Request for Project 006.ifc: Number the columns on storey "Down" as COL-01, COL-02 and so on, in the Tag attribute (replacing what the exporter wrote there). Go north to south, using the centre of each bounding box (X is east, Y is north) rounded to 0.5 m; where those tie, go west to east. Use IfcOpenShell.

First a look at what the model holds.

```python
import ifcopenshell
import ifcopenshell.util.element
import ifcopenshell.util.placement

model = ifcopenshell.open("Project 006.ifc")
print(model.schema)
storey = next(s for s in model.by_type("IfcBuildingStorey") if s.Name == "Down")
columns = [e for e in ifcopenshell.util.element.get_decomposition(storey) if e.is_a("IfcColumn")]
for e in sorted(columns, key=lambda e: e.id()):
    origin = ifcopenshell.util.placement.get_local_placement(e.ObjectPlacement)[:3, 3]
    print(e.id(), e.Tag, e.Name, origin.round(2) + 0.0, sep=" | ")
```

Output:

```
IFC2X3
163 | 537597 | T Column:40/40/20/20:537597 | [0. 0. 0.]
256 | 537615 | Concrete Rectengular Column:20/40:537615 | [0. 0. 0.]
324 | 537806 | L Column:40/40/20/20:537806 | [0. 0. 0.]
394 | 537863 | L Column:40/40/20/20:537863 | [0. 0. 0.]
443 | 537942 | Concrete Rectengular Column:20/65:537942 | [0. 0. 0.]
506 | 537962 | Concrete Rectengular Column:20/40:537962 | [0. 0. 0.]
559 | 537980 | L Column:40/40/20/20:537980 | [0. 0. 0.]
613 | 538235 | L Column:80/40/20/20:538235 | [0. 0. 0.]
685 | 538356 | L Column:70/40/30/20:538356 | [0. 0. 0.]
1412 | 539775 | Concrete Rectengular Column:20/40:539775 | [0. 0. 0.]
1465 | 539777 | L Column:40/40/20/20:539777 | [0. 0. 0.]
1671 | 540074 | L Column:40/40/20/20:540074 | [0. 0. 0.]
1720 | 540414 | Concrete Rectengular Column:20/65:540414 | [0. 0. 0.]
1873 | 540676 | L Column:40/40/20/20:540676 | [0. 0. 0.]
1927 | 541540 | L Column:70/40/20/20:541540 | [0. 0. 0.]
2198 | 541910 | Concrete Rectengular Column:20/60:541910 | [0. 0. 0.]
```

```python
import ifcopenshell
import ifcopenshell.geom
import ifcopenshell.util.element
import ifcopenshell.util.shape

model = ifcopenshell.open("Project 006.ifc")
settings = ifcopenshell.geom.settings()
settings.set("use-world-coords", True)


def centre(element):
    shape = ifcopenshell.geom.create_shape(settings, element)
    return ifcopenshell.util.shape.get_bbox_centroid(shape.geometry)


storey = next(s for s in model.by_type("IfcBuildingStorey") if s.Name == "Down")
columns = [e for e in ifcopenshell.util.element.get_decomposition(storey) if e.is_a("IfcColumn")]

# Insertion points can sit at a corner or the storey origin, so sort by the geometry (in metres).
centres = {e: centre(e) for e in columns}
columns.sort(key=lambda e: (-round(centres[e][1] / 0.5), centres[e][0]))

for i, e in enumerate(columns, start=1):
    number = f"COL-{i:02d}"
    e.Tag = number
    print(e.id(), number)

model.write("Project 006_edited.ifc")
```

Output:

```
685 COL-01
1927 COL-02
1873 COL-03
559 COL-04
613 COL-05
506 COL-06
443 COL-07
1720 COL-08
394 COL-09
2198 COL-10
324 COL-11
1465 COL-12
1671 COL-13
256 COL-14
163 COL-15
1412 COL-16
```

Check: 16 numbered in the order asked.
